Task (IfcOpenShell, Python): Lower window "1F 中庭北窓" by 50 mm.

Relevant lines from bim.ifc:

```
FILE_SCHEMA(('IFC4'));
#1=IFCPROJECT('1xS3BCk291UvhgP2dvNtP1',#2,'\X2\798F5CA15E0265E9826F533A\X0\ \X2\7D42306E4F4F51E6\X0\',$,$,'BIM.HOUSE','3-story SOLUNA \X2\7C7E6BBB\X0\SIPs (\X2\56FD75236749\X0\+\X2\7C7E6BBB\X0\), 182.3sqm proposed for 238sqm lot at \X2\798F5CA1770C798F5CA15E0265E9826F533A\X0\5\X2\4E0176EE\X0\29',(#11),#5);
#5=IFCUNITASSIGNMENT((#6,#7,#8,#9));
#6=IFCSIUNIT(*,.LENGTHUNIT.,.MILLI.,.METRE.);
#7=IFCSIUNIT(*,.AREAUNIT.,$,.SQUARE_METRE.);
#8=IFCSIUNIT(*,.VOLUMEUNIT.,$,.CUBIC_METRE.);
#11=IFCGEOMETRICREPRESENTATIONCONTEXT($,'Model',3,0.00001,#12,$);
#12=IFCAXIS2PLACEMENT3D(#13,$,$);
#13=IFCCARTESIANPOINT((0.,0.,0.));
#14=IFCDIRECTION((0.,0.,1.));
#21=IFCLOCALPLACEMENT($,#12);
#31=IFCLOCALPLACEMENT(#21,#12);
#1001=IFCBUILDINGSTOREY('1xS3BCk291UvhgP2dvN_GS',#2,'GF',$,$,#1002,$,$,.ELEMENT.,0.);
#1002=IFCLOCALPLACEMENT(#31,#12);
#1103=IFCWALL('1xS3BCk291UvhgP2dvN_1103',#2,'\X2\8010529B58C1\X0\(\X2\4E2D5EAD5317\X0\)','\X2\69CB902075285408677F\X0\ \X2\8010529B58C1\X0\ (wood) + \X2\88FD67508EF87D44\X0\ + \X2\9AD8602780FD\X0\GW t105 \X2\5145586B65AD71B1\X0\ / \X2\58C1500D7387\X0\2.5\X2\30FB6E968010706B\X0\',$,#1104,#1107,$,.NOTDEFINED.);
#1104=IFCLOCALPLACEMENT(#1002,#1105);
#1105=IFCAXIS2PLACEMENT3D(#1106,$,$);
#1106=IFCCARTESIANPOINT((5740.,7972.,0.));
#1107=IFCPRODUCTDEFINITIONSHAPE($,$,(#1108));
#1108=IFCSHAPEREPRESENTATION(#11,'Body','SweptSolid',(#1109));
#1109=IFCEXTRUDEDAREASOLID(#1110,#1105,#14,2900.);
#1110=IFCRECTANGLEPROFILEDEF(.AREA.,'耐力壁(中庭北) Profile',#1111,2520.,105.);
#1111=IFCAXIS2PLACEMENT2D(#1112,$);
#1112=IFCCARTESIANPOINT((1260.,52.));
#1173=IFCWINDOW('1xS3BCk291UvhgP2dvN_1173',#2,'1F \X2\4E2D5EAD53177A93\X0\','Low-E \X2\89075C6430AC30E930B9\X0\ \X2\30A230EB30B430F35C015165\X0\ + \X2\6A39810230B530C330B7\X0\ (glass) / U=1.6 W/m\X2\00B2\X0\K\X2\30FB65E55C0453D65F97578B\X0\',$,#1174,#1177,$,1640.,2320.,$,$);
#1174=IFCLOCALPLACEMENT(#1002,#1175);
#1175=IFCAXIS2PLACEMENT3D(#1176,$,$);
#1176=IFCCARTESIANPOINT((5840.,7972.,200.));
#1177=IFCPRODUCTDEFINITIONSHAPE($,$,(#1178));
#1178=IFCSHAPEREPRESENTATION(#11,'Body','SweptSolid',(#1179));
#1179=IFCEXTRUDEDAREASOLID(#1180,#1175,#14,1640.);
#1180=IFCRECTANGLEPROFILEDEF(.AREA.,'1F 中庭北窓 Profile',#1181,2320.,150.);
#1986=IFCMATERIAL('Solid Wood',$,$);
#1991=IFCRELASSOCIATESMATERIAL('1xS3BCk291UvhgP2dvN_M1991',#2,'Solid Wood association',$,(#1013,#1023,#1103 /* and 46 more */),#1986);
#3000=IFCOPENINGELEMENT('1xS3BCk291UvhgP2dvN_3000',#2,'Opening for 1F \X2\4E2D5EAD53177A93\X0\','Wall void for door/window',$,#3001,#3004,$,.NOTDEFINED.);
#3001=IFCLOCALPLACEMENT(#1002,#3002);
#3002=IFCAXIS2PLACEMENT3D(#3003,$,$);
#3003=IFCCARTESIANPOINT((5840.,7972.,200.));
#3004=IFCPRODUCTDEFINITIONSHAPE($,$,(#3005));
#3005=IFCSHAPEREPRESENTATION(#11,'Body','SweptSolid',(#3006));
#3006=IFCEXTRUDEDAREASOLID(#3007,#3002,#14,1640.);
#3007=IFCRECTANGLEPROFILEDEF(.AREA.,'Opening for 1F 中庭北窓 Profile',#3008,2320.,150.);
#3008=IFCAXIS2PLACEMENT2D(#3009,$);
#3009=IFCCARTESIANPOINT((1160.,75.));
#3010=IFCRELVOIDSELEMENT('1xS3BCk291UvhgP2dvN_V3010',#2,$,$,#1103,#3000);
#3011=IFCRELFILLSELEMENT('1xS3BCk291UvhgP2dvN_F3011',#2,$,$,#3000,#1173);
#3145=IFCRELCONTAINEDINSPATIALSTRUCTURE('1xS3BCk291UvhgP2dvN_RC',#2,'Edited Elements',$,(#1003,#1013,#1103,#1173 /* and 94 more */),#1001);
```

```python
import numpy as np
import ifcopenshell
import ifcopenshell.api.geometry
import ifcopenshell.util.placement
import ifcopenshell.util.unit

model = ifcopenshell.open("bim.ifc")
unit_scale = ifcopenshell.util.unit.calculate_unit_scale(model)

window = model.by_guid("1xS3BCk291UvhgP2dvN_1173")
opening = window.FillsVoids[0].RelatingOpeningElement
dz = -0.05 / unit_scale

shift = np.array([0.0, 0.0, dz])
# The window is not placed relative to its opening, so move both.
for product in (opening, window):
    matrix = ifcopenshell.util.placement.get_local_placement(product.ObjectPlacement)
    matrix[:3, 3] += shift
    ifcopenshell.api.geometry.edit_object_placement(model, product=product, matrix=matrix, is_si=False)

print(f"moved by {dz * unit_scale:+.3f} m")

model.write("bim_updated.ifc")
```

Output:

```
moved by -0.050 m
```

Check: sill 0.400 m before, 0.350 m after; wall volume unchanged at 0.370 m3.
